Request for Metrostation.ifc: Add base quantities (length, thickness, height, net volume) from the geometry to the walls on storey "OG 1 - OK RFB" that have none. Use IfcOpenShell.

First a look at what the model holds.

```python
import ifcopenshell
import ifcopenshell.util.element
import ifcopenshell.util.unit

model = ifcopenshell.open("Metrostation.ifc")
print(model.schema)
for unit_type in ("LENGTHUNIT", "AREAUNIT", "VOLUMEUNIT"):
    print(unit_type, ifcopenshell.util.unit.calculate_unit_scale(model, unit_type))
storey = next(s for s in model.by_type("IfcBuildingStorey") if s.Name == "OG 1 - OK RFB")
walls = [e for e in ifcopenshell.util.element.get_decomposition(storey) if e.is_a("IfcWall")]
for e in sorted(walls, key=lambda e: e.id()):
    print(e.id(), e.is_a(), e.Name, list(ifcopenshell.util.element.get_psets(e, qtos_only=True)), sep=" | ")
```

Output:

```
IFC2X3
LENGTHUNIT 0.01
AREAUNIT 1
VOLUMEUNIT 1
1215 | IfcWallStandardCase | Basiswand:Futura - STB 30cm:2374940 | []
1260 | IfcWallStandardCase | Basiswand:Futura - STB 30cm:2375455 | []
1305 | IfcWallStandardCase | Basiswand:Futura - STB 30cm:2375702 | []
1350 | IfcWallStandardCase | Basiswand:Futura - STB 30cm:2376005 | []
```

```python
import ifcopenshell
import ifcopenshell.api.pset
import ifcopenshell.geom
import ifcopenshell.util.element
import ifcopenshell.util.shape
import ifcopenshell.util.unit

model = ifcopenshell.open("Metrostation.ifc")
unit_scale = ifcopenshell.util.unit.calculate_unit_scale(model)
volume_scale = ifcopenshell.util.unit.calculate_unit_scale(model, "VOLUMEUNIT")
settings = ifcopenshell.geom.settings()

storey = next(s for s in model.by_type("IfcBuildingStorey") if s.Name == "OG 1 - OK RFB")
walls = [e for e in ifcopenshell.util.element.get_decomposition(storey) if e.is_a("IfcWall")]

for e in sorted(walls, key=lambda e: e.id()):
    if ifcopenshell.util.element.get_psets(e, qtos_only=True, should_inherit=False):
        continue
    # Geometry comes back in metres, in the element's own axes.
    shape = ifcopenshell.geom.create_shape(settings, e)
    values = {
        "Length": ifcopenshell.util.shape.get_x(shape.geometry) / unit_scale,
        "Width": ifcopenshell.util.shape.get_y(shape.geometry) / unit_scale,
        "Height": ifcopenshell.util.shape.get_z(shape.geometry) / unit_scale,
        "NetVolume": ifcopenshell.util.shape.get_volume(shape.geometry) / volume_scale,
    }
    qto = ifcopenshell.api.pset.add_qto(model, product=e, name="BaseQuantities")
    ifcopenshell.api.pset.edit_qto(model, qto=qto, properties=values)
    print(e.id(), {k: round(v, 3) for k, v in values.items()})

model.write("Metrostation_v2.ifc")
```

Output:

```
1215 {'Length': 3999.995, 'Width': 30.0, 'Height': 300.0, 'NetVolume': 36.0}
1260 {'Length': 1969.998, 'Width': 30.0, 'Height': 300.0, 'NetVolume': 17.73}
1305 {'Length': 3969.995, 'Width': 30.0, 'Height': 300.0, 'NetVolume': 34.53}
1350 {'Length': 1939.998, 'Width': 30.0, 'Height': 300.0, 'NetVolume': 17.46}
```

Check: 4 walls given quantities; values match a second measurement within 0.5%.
